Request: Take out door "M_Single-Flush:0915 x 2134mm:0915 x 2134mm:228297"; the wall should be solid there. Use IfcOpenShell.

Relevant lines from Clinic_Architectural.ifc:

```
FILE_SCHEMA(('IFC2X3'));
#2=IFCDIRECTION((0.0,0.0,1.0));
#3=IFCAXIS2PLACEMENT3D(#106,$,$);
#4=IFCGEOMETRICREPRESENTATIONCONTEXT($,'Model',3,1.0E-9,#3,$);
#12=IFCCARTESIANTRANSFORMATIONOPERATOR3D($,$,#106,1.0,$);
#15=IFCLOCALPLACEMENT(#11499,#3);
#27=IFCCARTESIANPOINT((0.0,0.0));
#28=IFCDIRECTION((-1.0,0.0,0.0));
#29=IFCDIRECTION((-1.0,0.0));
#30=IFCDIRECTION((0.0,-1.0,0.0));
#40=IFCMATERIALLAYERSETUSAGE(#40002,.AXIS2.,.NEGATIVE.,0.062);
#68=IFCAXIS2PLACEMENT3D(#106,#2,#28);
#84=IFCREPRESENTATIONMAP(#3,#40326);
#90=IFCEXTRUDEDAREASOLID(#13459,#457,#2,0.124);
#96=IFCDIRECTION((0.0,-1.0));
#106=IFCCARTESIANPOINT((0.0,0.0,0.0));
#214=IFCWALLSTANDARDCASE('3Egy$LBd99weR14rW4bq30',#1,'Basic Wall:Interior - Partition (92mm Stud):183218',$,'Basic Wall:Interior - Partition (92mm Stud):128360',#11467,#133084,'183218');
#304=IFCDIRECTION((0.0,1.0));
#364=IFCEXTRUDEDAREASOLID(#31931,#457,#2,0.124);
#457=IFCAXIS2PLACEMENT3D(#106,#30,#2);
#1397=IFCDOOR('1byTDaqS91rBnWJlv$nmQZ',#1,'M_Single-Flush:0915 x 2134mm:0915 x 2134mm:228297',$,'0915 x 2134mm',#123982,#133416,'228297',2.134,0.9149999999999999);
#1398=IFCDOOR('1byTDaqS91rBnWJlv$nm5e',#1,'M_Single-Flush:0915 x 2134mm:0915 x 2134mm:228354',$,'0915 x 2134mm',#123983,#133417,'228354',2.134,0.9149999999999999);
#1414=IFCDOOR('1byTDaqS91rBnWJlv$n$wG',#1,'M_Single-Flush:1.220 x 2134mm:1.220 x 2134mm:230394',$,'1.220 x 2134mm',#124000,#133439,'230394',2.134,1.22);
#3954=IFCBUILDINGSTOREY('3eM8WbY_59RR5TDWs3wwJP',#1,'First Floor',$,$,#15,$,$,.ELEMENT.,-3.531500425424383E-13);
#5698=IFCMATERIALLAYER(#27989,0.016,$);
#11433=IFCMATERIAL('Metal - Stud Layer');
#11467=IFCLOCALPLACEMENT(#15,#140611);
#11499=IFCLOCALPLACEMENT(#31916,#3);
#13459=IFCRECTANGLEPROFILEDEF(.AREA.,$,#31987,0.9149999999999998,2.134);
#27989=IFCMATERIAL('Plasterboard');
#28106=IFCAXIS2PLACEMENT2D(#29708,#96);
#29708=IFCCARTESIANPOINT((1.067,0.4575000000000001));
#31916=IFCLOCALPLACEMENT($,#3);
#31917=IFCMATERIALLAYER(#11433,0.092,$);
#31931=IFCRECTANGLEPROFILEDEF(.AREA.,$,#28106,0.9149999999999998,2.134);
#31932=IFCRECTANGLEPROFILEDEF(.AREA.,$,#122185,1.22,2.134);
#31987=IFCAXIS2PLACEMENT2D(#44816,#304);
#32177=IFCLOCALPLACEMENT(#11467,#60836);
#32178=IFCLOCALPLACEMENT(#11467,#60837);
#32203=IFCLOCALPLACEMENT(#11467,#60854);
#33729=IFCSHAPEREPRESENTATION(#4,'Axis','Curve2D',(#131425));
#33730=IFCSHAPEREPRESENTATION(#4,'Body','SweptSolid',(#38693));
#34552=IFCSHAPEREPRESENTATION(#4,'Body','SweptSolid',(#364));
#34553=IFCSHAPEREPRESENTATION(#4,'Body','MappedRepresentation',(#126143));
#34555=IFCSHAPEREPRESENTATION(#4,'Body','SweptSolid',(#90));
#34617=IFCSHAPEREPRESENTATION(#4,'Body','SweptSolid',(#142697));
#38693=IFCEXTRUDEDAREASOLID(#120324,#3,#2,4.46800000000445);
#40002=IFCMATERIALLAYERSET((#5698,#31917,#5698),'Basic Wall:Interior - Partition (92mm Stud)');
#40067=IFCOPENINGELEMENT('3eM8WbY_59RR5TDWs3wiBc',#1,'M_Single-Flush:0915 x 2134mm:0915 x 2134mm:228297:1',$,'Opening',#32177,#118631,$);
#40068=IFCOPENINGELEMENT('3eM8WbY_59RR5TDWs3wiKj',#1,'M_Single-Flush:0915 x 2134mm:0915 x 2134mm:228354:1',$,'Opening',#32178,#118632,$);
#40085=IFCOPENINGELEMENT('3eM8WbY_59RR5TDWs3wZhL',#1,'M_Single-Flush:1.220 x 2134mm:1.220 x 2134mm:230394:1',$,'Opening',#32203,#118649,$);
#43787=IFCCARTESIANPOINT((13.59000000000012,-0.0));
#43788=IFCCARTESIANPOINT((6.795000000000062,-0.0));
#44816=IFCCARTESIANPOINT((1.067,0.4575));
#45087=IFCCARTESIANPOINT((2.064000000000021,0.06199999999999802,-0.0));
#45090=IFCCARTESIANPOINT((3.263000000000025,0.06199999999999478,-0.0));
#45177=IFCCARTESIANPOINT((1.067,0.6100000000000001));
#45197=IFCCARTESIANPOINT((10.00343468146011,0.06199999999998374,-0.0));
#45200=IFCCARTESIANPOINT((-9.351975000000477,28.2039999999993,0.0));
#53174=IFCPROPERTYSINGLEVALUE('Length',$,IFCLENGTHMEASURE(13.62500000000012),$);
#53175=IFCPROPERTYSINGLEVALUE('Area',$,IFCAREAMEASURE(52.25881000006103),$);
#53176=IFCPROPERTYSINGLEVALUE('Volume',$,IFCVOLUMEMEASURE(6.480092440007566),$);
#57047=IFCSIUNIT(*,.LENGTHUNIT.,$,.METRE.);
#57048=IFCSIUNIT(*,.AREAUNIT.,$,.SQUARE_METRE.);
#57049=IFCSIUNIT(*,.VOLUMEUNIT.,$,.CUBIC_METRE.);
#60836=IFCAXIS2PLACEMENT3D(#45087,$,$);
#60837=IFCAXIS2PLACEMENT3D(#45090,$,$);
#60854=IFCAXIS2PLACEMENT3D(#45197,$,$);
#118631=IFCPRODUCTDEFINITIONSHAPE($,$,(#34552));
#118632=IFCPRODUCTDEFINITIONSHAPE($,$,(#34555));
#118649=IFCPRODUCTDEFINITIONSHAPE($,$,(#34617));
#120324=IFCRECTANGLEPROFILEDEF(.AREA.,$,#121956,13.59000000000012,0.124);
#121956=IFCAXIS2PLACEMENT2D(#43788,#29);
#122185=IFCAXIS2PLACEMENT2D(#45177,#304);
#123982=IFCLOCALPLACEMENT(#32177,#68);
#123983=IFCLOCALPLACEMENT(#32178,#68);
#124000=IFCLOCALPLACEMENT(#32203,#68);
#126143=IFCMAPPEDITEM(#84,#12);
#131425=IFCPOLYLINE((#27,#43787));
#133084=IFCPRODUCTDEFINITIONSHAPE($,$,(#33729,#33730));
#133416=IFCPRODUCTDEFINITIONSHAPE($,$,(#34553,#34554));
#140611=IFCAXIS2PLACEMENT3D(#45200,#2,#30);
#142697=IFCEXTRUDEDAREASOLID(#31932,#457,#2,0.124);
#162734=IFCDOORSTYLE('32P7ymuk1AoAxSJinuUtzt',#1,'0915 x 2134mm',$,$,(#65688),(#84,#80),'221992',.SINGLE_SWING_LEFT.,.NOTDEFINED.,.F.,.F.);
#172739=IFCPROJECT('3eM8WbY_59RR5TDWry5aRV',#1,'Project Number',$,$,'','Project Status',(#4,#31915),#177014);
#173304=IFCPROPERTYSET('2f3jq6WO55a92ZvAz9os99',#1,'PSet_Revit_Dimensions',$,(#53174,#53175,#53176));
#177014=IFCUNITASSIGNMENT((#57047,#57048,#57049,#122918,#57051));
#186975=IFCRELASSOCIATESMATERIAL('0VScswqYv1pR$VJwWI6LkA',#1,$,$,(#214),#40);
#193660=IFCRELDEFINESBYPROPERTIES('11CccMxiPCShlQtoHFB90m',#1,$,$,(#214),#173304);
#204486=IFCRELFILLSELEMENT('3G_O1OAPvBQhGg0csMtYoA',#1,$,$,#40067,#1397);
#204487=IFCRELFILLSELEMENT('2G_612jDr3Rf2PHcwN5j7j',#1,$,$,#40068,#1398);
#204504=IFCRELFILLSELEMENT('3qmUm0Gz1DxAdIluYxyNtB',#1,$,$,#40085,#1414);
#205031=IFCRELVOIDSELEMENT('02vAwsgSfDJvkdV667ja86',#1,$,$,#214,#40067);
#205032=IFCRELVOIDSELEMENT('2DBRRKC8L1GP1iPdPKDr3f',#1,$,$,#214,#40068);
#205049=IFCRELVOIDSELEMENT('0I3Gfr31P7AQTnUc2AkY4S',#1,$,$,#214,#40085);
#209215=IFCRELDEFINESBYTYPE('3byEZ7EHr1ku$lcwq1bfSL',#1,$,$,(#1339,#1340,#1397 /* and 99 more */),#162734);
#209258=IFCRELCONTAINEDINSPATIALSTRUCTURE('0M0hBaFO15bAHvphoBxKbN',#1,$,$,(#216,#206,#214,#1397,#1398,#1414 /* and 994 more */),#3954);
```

```python
import ifcopenshell
import ifcopenshell.api.feature
import ifcopenshell.api.pset
import ifcopenshell.api.root
import ifcopenshell.geom
import ifcopenshell.util.element
import ifcopenshell.util.shape
import ifcopenshell.util.unit

model = ifcopenshell.open("Clinic_Architectural.ifc")
area_scale = ifcopenshell.util.unit.calculate_unit_scale(model, "AREAUNIT")
volume_scale = ifcopenshell.util.unit.calculate_unit_scale(model, "VOLUMEUNIT")
settings = ifcopenshell.geom.settings()


def volume(element):
    """Net volume in cubic metres, openings subtracted."""
    shape = ifcopenshell.geom.create_shape(settings, element)
    return ifcopenshell.util.shape.get_volume(shape.geometry)


door = model.by_guid("1byTDaqS91rBnWJlv$nmQZ")
opening = door.FillsVoids[0].RelatingOpeningElement
wall = opening.VoidsElements[0].RelatingBuildingElement
before = volume(wall)

ifcopenshell.api.root.remove_product(model, product=door)
ifcopenshell.api.feature.remove_feature(model, feature=opening)

after = volume(wall)
thickness = 0.124  # wall thickness in metres

# Update the wall's stored quantities.
pset = model.by_id(ifcopenshell.util.element.get_pset(wall, "PSet_Revit_Dimensions", should_inherit=False)["id"])
ifcopenshell.api.pset.edit_pset(model, pset=pset, properties={
    "Area": model.create_entity("IfcAreaMeasure", after / thickness / area_scale),
    "Volume": model.create_entity("IfcVolumeMeasure", after / volume_scale),
})

print(f"wall volume {before:.3f} -> {after:.3f} m3")

model.write("Clinic_Architectural_updated.ifc")
```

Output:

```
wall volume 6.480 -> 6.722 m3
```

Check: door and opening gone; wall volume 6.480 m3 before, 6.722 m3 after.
